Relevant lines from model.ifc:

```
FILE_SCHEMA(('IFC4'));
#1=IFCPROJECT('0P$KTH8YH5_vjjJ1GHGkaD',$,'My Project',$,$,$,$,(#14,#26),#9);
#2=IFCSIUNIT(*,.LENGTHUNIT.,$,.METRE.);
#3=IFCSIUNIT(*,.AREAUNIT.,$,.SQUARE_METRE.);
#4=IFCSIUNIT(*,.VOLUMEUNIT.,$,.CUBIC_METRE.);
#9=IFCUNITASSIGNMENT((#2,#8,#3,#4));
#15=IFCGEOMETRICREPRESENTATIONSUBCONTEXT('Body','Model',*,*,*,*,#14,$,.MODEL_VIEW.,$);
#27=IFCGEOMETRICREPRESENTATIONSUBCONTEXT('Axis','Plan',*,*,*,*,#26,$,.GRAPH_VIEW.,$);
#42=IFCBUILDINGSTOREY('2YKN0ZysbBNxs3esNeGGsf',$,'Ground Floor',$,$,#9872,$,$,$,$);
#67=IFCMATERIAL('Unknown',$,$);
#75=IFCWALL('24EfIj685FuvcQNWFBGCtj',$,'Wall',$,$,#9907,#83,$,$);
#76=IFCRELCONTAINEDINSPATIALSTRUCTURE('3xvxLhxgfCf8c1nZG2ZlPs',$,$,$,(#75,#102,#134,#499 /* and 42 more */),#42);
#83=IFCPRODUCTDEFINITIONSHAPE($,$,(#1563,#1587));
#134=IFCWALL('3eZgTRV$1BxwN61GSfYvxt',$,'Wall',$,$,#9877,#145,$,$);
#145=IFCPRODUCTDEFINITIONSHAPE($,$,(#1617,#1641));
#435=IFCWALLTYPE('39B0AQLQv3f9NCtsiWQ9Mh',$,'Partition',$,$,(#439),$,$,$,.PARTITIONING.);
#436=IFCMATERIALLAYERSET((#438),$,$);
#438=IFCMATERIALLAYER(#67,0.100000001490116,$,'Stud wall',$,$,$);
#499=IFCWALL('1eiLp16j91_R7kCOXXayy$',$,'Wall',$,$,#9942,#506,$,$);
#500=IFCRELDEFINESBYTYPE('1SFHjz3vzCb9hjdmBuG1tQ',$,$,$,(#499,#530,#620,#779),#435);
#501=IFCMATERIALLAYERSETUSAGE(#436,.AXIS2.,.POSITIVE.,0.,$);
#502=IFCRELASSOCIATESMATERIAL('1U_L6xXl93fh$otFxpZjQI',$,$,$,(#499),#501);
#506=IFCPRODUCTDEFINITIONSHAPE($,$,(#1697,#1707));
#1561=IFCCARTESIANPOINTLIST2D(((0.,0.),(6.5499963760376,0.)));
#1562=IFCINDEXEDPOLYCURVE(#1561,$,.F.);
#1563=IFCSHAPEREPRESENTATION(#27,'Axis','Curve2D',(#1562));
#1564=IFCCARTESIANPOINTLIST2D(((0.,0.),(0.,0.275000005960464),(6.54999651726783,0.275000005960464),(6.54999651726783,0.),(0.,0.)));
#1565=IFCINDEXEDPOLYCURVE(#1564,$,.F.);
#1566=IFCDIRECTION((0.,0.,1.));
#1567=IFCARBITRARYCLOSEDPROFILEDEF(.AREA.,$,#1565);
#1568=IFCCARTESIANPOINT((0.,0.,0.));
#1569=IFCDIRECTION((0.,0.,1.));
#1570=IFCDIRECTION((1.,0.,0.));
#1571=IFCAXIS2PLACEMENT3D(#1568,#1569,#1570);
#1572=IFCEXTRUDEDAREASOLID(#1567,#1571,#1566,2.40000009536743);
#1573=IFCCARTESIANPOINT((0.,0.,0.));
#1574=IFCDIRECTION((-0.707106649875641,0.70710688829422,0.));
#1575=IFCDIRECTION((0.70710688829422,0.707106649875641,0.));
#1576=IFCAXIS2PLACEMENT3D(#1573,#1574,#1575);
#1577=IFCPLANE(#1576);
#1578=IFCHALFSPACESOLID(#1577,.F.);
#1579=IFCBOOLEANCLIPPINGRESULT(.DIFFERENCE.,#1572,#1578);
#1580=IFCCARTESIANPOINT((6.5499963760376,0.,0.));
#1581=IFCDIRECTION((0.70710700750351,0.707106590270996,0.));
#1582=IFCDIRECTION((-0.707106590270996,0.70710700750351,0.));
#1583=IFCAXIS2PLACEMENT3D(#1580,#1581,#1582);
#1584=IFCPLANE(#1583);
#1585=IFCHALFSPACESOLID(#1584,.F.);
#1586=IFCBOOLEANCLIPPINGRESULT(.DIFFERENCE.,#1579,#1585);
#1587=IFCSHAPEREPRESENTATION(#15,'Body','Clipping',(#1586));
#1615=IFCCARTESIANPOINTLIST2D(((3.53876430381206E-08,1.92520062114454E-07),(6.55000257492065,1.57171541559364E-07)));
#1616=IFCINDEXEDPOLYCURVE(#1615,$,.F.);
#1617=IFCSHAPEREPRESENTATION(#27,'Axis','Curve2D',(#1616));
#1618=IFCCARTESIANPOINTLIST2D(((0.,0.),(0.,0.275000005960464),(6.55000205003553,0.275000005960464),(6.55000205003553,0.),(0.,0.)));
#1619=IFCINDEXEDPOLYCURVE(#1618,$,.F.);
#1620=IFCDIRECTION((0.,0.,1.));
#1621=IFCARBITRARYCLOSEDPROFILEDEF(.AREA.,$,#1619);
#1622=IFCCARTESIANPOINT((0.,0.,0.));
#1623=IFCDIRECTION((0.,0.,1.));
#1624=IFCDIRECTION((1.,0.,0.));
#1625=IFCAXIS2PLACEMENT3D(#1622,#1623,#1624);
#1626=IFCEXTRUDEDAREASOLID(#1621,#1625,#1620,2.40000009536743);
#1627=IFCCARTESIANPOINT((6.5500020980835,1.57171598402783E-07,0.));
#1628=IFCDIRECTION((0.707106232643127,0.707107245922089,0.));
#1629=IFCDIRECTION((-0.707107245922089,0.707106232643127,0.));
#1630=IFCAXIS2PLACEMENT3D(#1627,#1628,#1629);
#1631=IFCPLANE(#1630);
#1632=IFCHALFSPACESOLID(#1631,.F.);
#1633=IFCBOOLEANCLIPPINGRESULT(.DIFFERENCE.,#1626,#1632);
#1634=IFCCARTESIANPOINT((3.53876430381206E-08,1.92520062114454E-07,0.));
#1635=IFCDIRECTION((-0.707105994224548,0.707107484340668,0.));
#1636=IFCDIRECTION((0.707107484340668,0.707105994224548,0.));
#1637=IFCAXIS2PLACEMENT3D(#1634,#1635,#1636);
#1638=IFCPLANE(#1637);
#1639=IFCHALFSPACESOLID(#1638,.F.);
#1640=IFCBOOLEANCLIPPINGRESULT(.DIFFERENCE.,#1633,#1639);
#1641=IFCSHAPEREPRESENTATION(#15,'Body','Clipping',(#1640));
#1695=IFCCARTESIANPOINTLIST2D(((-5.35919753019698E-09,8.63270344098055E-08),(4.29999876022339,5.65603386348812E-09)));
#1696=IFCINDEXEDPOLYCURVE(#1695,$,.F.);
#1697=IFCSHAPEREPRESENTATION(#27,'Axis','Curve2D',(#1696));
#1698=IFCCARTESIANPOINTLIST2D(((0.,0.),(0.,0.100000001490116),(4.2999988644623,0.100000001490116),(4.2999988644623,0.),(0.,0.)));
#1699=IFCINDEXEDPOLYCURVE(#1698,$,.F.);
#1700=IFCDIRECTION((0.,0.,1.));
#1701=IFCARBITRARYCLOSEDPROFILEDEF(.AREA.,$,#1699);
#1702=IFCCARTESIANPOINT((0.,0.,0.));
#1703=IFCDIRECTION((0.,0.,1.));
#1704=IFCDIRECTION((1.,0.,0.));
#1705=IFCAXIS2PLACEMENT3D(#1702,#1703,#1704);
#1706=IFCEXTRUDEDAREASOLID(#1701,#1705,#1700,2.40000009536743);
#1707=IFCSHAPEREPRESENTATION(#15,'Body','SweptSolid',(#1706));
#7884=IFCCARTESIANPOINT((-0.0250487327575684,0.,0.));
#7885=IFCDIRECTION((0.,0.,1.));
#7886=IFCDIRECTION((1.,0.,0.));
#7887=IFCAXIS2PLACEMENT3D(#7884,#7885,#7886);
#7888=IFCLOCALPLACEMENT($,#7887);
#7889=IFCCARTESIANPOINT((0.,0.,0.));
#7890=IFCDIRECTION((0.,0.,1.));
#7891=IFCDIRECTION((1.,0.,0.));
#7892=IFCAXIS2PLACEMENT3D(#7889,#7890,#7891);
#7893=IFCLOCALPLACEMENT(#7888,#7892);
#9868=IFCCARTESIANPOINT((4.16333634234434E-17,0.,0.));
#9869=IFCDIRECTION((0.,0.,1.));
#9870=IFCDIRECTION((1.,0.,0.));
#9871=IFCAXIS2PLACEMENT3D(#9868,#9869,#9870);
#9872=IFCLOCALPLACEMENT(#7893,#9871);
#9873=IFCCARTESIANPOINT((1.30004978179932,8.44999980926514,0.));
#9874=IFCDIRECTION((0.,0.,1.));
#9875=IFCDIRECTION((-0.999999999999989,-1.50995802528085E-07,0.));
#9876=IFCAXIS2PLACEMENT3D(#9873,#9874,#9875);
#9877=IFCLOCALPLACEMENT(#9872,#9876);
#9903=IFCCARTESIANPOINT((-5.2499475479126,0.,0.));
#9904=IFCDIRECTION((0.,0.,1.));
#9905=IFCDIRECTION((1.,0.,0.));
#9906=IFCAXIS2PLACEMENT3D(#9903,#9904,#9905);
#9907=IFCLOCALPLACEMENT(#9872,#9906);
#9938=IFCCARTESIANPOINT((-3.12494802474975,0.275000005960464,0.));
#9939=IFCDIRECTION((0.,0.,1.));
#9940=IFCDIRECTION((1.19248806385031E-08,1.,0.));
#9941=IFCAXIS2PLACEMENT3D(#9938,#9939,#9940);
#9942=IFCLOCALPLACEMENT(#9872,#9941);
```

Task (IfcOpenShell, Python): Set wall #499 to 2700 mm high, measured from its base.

```python
import ifcopenshell
import ifcopenshell.geom
import ifcopenshell.util.representation
import ifcopenshell.util.shape
import ifcopenshell.util.unit

model = ifcopenshell.open("model.ifc")
unit_scale = ifcopenshell.util.unit.calculate_unit_scale(model)
settings = ifcopenshell.geom.settings()


def volume(element):
    """Net volume in cubic metres, openings subtracted."""
    shape = ifcopenshell.geom.create_shape(settings, element)
    return ifcopenshell.util.shape.get_volume(shape.geometry)


wall = model.by_guid("1eiLp16j91_R7kCOXXayy$")
before = volume(wall)

body = ifcopenshell.util.representation.get_representation(wall, "Model", "Body")
solid = body.Items[0]
old_height = solid.Depth
solid.Depth = 2.7 / unit_scale
after = volume(wall)

print(f"height {old_height:g} -> {solid.Depth:g}, volume {before:.3f} -> {after:.3f} m3")

model.write("model_edited.ifc")
```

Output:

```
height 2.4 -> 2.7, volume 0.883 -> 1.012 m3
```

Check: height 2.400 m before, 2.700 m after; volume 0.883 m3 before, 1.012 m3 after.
